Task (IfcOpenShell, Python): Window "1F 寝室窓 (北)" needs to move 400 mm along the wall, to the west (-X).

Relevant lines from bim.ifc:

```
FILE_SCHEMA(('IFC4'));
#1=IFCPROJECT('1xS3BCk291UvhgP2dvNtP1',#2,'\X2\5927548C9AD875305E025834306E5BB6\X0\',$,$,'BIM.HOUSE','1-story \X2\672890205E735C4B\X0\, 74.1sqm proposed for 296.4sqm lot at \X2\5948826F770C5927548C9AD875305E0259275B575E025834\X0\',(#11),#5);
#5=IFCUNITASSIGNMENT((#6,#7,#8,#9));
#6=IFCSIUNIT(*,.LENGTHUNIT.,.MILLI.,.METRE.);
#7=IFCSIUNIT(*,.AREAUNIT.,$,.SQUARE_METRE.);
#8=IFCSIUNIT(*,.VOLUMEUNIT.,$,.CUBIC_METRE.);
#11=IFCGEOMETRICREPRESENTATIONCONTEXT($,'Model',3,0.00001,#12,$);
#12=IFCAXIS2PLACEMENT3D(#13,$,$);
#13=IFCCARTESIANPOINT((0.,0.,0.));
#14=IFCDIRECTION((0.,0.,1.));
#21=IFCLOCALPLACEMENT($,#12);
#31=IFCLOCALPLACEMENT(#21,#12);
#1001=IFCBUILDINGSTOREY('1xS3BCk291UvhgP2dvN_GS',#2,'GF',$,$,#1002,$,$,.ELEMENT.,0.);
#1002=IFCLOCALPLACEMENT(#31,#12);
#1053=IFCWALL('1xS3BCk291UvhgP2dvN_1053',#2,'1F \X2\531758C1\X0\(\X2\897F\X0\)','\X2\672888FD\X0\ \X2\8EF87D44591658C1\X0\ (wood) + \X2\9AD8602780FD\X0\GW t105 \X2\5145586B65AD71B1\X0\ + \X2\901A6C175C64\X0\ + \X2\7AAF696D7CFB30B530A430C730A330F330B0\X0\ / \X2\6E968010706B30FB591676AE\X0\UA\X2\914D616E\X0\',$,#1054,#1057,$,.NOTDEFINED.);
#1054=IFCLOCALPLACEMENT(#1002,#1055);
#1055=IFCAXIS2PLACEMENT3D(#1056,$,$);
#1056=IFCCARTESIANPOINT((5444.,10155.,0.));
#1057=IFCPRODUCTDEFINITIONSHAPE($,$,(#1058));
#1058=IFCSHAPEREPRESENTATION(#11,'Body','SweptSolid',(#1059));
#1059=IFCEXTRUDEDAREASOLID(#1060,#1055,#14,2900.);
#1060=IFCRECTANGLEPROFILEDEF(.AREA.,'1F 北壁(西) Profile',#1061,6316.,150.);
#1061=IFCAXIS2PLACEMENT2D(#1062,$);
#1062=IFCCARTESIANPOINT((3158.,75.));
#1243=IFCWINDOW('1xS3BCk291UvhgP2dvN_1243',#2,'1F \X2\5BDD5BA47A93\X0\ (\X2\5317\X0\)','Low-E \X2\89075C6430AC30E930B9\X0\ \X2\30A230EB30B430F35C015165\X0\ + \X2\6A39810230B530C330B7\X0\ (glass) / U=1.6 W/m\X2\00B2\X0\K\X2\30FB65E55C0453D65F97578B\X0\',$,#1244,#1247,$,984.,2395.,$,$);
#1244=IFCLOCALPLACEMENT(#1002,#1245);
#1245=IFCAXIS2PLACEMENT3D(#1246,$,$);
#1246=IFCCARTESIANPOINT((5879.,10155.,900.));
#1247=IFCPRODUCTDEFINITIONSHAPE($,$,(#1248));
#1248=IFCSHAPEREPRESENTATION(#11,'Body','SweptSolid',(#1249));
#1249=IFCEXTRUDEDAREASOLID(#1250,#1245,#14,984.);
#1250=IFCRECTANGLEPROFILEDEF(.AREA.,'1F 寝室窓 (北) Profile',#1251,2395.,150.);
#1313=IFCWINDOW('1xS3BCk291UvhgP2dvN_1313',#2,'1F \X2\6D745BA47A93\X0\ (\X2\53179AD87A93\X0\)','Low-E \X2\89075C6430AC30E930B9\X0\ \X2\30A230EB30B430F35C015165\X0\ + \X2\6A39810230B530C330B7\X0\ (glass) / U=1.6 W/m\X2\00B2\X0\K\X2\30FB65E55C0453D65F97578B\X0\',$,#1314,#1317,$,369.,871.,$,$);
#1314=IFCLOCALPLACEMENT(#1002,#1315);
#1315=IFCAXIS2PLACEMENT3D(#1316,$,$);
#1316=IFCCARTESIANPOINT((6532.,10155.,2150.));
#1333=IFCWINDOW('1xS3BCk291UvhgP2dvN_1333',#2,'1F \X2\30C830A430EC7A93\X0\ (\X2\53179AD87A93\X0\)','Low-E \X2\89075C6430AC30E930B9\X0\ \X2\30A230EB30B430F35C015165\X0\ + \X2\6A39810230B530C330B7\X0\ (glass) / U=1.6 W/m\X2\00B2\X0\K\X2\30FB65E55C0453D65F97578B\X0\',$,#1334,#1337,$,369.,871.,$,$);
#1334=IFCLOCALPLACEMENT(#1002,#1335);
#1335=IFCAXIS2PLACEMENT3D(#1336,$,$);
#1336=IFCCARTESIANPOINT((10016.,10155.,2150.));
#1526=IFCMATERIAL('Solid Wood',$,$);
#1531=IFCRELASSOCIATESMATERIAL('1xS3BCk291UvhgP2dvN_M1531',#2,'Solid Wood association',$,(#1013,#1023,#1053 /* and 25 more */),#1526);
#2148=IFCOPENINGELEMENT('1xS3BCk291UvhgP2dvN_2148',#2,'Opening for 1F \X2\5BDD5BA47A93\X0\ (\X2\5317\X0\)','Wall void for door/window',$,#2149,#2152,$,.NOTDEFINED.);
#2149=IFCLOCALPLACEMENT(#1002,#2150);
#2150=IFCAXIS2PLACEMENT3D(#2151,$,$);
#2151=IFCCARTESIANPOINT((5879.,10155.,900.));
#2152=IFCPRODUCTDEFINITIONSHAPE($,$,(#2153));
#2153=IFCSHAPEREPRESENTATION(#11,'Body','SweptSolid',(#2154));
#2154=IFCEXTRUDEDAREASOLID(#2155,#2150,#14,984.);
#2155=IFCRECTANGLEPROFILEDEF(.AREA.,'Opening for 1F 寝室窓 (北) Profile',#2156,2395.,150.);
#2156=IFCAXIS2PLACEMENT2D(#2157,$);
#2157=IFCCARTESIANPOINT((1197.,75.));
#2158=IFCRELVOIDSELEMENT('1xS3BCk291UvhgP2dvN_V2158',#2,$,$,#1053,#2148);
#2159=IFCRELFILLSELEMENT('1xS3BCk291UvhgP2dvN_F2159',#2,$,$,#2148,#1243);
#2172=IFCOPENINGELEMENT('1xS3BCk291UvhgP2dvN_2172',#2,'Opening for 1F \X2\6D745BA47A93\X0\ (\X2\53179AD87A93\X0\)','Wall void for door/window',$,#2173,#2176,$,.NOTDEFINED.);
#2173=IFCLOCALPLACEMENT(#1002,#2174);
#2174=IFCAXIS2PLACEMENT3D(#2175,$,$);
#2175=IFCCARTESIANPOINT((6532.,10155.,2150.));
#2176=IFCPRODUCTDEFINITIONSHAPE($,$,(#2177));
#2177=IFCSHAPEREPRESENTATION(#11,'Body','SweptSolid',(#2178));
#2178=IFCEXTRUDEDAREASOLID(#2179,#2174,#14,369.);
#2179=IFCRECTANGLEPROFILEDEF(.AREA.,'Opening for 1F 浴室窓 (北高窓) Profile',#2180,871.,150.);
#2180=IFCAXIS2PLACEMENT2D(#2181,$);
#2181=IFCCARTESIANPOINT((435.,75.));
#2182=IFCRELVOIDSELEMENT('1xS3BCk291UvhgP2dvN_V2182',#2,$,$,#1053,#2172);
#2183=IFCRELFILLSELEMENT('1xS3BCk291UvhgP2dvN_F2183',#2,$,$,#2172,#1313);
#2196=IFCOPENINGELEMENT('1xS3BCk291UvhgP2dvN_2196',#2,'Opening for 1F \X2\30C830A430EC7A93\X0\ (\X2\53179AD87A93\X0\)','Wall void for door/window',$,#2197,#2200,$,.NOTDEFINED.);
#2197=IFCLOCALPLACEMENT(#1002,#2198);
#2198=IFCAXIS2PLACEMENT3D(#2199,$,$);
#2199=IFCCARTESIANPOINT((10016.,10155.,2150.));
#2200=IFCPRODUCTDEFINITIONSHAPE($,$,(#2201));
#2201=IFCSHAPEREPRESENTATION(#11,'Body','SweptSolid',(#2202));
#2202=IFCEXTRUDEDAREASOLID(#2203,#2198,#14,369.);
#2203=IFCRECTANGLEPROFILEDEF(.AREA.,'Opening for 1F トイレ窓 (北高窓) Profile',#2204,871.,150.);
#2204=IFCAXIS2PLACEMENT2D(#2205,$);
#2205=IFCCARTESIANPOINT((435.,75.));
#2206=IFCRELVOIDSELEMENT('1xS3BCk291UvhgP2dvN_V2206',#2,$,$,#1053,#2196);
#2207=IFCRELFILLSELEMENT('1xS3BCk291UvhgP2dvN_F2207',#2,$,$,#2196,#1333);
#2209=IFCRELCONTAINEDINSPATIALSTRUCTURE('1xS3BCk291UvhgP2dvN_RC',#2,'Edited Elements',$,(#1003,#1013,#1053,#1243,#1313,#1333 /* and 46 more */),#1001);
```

```python
import ifcopenshell
import ifcopenshell.api.geometry
import ifcopenshell.util.placement

model = ifcopenshell.open("bim.ifc")

window = model.by_guid("1xS3BCk291UvhgP2dvN_1243")
opening = window.FillsVoids[0].RelatingOpeningElement
wall = opening.VoidsElements[0].RelatingBuildingElement

wall_matrix = ifcopenshell.util.placement.get_local_placement(wall.ObjectPlacement)
shift = wall_matrix[:3, 0] * -400.0
before = ifcopenshell.util.placement.get_local_placement(window.ObjectPlacement)[:3, 3].copy()

# The window is not placed relative to its opening, so move both.
for product in (opening, window):
    matrix = ifcopenshell.util.placement.get_local_placement(product.ObjectPlacement)
    matrix[:3, 3] += shift
    ifcopenshell.api.geometry.edit_object_placement(model, product=product, matrix=matrix, is_si=False)

after = ifcopenshell.util.placement.get_local_placement(window.ObjectPlacement)[:3, 3]
print("window moved by", (after - before).round(3) + 0.0)

model.write("bim_updated.ifc")
```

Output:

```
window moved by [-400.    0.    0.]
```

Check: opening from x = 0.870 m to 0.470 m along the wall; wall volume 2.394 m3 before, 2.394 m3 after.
